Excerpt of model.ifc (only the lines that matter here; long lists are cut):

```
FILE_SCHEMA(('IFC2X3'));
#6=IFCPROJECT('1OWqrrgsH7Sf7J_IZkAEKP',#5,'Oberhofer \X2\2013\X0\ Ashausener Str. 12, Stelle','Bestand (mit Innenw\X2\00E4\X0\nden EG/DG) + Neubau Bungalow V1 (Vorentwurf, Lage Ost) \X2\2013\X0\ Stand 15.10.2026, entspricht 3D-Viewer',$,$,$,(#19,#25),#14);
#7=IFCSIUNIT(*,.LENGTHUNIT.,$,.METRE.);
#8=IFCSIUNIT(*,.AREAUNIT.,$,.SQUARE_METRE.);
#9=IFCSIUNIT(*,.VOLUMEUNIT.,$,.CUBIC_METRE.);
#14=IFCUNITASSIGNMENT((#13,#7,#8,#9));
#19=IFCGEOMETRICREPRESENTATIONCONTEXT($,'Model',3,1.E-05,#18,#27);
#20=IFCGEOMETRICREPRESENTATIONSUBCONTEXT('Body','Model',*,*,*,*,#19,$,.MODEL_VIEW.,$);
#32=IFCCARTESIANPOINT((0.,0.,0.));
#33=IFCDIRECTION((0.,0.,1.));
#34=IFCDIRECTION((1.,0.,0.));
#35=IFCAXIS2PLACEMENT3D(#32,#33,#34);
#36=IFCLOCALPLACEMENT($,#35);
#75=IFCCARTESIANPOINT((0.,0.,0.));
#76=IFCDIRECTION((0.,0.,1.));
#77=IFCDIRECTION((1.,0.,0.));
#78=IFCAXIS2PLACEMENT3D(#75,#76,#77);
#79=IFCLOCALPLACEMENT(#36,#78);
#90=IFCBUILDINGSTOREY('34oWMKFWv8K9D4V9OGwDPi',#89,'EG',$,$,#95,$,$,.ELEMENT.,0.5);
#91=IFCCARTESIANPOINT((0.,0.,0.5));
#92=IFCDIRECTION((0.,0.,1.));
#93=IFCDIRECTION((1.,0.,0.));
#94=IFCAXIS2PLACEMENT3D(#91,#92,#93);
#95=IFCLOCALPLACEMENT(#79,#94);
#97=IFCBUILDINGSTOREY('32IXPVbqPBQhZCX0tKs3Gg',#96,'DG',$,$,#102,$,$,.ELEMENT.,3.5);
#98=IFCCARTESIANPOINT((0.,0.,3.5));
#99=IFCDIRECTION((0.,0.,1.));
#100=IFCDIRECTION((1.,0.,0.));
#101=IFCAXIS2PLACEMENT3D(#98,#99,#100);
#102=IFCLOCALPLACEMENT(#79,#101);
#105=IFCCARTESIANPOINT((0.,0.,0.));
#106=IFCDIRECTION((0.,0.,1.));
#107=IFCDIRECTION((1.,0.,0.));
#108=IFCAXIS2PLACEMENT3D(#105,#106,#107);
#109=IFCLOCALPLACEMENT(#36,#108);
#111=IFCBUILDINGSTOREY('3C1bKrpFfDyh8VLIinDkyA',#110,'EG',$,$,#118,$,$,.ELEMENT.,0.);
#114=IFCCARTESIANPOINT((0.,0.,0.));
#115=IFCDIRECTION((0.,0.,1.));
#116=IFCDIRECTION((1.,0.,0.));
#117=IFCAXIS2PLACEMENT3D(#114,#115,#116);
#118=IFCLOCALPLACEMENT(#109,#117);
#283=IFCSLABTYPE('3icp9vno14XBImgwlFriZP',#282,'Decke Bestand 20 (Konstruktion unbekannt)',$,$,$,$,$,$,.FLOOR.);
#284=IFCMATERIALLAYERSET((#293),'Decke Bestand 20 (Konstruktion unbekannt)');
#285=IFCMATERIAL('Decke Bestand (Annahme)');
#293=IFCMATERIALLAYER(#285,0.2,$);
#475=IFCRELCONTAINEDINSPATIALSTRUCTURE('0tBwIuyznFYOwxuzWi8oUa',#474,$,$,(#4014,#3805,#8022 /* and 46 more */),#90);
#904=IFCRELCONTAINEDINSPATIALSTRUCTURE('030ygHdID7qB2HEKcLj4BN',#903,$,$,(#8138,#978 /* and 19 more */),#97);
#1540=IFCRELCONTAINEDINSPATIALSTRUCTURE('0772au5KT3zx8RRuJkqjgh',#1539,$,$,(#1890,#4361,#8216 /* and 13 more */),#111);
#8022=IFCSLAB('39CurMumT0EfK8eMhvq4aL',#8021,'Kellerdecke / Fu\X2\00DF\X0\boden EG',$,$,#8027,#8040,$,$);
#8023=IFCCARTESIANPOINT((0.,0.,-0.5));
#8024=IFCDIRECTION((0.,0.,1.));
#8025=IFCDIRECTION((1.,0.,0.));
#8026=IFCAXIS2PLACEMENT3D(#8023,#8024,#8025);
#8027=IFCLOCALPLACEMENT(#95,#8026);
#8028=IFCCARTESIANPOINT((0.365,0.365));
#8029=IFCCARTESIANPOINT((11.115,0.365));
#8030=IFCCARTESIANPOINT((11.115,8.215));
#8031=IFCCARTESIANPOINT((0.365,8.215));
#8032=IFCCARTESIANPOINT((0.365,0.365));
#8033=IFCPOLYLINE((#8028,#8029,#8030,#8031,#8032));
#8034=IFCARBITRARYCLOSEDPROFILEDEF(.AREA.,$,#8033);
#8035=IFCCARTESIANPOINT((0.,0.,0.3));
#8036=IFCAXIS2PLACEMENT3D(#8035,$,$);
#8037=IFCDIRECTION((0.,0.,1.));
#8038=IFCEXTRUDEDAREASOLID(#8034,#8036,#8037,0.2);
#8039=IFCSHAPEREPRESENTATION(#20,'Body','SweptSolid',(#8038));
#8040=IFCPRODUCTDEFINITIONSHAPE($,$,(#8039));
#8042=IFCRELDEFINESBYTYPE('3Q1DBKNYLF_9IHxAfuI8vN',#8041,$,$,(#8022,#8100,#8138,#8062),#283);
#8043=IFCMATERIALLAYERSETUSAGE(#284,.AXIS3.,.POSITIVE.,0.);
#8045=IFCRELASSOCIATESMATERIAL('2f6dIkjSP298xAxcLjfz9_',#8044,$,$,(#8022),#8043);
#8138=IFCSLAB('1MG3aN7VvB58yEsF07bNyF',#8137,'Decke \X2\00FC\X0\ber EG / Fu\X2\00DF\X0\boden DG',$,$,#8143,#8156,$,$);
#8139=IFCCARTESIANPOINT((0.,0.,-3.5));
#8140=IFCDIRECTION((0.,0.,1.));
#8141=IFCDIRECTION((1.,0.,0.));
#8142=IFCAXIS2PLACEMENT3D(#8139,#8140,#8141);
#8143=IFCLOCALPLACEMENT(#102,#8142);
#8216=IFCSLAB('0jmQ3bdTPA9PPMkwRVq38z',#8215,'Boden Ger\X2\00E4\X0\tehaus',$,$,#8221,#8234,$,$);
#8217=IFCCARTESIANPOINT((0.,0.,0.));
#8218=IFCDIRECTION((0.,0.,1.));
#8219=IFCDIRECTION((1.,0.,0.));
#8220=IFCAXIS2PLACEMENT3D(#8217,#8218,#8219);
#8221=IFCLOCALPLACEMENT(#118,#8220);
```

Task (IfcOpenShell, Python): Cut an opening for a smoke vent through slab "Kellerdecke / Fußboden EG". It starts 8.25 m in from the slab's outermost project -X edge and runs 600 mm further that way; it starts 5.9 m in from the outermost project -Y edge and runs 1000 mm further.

```python
import numpy as np
import ifcopenshell
import ifcopenshell.api.feature
import ifcopenshell.api.geometry
import ifcopenshell.api.root
import ifcopenshell.geom
import ifcopenshell.util.placement
import ifcopenshell.util.representation
import ifcopenshell.util.shape
import ifcopenshell.util.unit

model = ifcopenshell.open("model.ifc")
unit_scale = ifcopenshell.util.unit.calculate_unit_scale(model)
settings = ifcopenshell.geom.settings()


def volume(element):
    """Net volume in cubic metres, openings subtracted."""
    shape = ifcopenshell.geom.create_shape(settings, element)
    return ifcopenshell.util.shape.get_volume(shape.geometry)


slab = model.by_id(8022)
before = volume(slab)

# Extent in the slab's own axes, in metres. The edges named are its -X and -Y sides.
slab_shape = ifcopenshell.geom.create_shape(settings, slab)
vertices = ifcopenshell.util.shape.get_vertices(slab_shape.geometry)
x_min, y_min, bottom = vertices.min(axis=0)
top = vertices[:, 2].max()

opening = ifcopenshell.api.root.create_entity(model, ifc_class="IfcOpeningElement", name="Smoke vent opening")
context = ifcopenshell.util.representation.get_context(model, "Model", "Body", "MODEL_VIEW")
width, depth = 0.6, 1
outline = [(0.0, 0.0), (width, 0.0), (width, depth), (0.0, depth), (0.0, 0.0)]
# Overshoot both faces by 50 mm so the cut is clean.
shape = ifcopenshell.api.geometry.add_slab_representation(
    model, context=context, depth=top - bottom + 0.1, polyline=outline
)
ifcopenshell.api.geometry.assign_representation(model, product=opening, representation=shape)

matrix = ifcopenshell.util.placement.get_local_placement(slab.ObjectPlacement)
matrix[:, 3] = matrix @ np.append(np.array([x_min + 8.25, y_min + 5.9, bottom - 0.05]) / unit_scale, 1.0)
ifcopenshell.api.geometry.edit_object_placement(model, product=opening, matrix=matrix, is_si=False)
ifcopenshell.api.feature.add_feature(model, feature=opening, element=slab)

after = volume(slab)

print(f"slab volume {before:.3f} -> {after:.3f} m3")

model.write("model_updated.ifc")
```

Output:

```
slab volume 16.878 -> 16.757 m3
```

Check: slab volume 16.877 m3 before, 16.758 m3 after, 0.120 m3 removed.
